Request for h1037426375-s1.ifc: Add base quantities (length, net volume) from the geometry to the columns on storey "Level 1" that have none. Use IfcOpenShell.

First a look at what the model holds.

```python
import ifcopenshell
import ifcopenshell.util.element
import ifcopenshell.util.unit

model = ifcopenshell.open("h1037426375-s1.ifc")
print(model.schema)
for unit_type in ("LENGTHUNIT", "AREAUNIT", "VOLUMEUNIT"):
    print(unit_type, ifcopenshell.util.unit.calculate_unit_scale(model, unit_type))
storey = next(s for s in model.by_type("IfcBuildingStorey") if s.Name == "Level 1")
columns = [e for e in ifcopenshell.util.element.get_decomposition(storey) if e.is_a("IfcColumn")]
for e in sorted(columns, key=lambda e: e.id()):
    print(e.id(), e.is_a(), e.Name, list(ifcopenshell.util.element.get_psets(e, qtos_only=True)), sep=" | ")
```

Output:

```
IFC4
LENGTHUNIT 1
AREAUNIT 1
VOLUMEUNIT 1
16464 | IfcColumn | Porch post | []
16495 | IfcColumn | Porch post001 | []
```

```python
import ifcopenshell
import ifcopenshell.api.pset
import ifcopenshell.geom
import ifcopenshell.util.element
import ifcopenshell.util.shape
import ifcopenshell.util.unit

model = ifcopenshell.open("h1037426375-s1.ifc")
unit_scale = ifcopenshell.util.unit.calculate_unit_scale(model)
volume_scale = ifcopenshell.util.unit.calculate_unit_scale(model, "VOLUMEUNIT")
settings = ifcopenshell.geom.settings()

storey = next(s for s in model.by_type("IfcBuildingStorey") if s.Name == "Level 1")
columns = [e for e in ifcopenshell.util.element.get_decomposition(storey) if e.is_a("IfcColumn")]

for e in sorted(columns, key=lambda e: e.id()):
    if ifcopenshell.util.element.get_psets(e, qtos_only=True, should_inherit=False):
        continue
    # Geometry comes back in metres, in the element's own axes.
    shape = ifcopenshell.geom.create_shape(settings, e)
    values = {
        "Length": ifcopenshell.util.shape.get_z(shape.geometry) / unit_scale,
        "NetVolume": ifcopenshell.util.shape.get_volume(shape.geometry) / volume_scale,
    }
    qto = ifcopenshell.api.pset.add_qto(model, product=e, name="Qto_ColumnBaseQuantities")
    ifcopenshell.api.pset.edit_qto(model, qto=qto, properties=values)
    print(e.id(), {k: round(v, 3) for k, v in values.items()})

model.write("h1037426375-s1-out.ifc")
```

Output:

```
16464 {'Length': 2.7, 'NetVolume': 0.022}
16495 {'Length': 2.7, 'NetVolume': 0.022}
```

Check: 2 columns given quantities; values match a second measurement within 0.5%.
